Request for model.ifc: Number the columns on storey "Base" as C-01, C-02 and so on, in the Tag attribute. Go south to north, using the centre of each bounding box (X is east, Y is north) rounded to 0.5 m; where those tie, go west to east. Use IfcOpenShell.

First a look at what the model holds.

```python
import ifcopenshell
import ifcopenshell.util.element
import ifcopenshell.util.placement

model = ifcopenshell.open("model.ifc")
print(model.schema)
storey = next(s for s in model.by_type("IfcBuildingStorey") if s.Name == "Base")
columns = [e for e in ifcopenshell.util.element.get_decomposition(storey) if e.is_a("IfcColumn")]
for e in sorted(columns, key=lambda e: e.id()):
    origin = ifcopenshell.util.placement.get_local_placement(e.ObjectPlacement)[:3, 3]
    print(e.id(), e.Tag, e.Name, origin.round(2) + 0.0, sep=" | ")
```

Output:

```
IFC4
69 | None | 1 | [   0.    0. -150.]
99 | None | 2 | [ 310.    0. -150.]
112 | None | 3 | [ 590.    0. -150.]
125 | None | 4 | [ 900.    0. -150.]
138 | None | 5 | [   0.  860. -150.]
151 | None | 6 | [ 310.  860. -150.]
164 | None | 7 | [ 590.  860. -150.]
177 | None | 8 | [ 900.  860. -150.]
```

```python
import ifcopenshell
import ifcopenshell.geom
import ifcopenshell.util.element
import ifcopenshell.util.shape

model = ifcopenshell.open("model.ifc")
settings = ifcopenshell.geom.settings()
settings.set("use-world-coords", True)


def centre(element):
    shape = ifcopenshell.geom.create_shape(settings, element)
    return ifcopenshell.util.shape.get_bbox_centroid(shape.geometry)


storey = next(s for s in model.by_type("IfcBuildingStorey") if s.Name == "Base")
columns = [e for e in ifcopenshell.util.element.get_decomposition(storey) if e.is_a("IfcColumn")]

# Insertion points can sit at a corner or the storey origin, so sort by the geometry (in metres).
centres = {e: centre(e) for e in columns}
columns.sort(key=lambda e: (round(centres[e][1] / 0.5), centres[e][0]))

for i, e in enumerate(columns, start=1):
    number = f"C-{i:02d}"
    e.Tag = number
    print(e.id(), number)

model.write("model_rev.ifc")
```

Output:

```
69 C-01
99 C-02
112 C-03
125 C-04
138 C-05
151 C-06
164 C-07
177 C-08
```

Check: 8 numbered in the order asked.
